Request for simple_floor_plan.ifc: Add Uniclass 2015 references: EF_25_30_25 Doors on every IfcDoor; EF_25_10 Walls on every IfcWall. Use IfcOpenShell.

First a look at what the model holds.

```python
import ifcopenshell

model = ifcopenshell.open("simple_floor_plan.ifc")
print(model.schema)
print("classifications:", [c.Name for c in model.by_type("IfcClassification")])
for ifc_class in ("IfcDoor", "IfcRoof", "IfcStair", "IfcWall", "IfcWindow"):
    print(ifc_class, len(model.by_type(ifc_class)))
```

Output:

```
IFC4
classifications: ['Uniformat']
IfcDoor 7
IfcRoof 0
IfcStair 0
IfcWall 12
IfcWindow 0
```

```python
import ifcopenshell
import ifcopenshell.api.classification

model = ifcopenshell.open("simple_floor_plan.ifc")

system = ifcopenshell.api.classification.add_classification(model, classification="Uniclass 2015")

codes = {
    "IfcDoor": ("EF_25_30_25", "Doors"),
    "IfcWall": ("EF_25_10", "Walls"),
}
for ifc_class, (code, name) in codes.items():
    products = model.by_type(ifc_class)
    ifcopenshell.api.classification.add_reference(
        model, products=products, classification=system, identification=code, name=name
    )
    print(code, len(products))

model.write("simple_floor_plan_v2.ifc")
```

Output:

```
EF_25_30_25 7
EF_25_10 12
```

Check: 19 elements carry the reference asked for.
